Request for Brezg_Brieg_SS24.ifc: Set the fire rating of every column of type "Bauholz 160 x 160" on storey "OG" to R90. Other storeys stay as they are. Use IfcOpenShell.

First a look at what the model holds.

```python
import ifcopenshell
import ifcopenshell.util.element

model = ifcopenshell.open("Brezg_Brieg_SS24.ifc")
print(model.schema)
storey = next(s for s in model.by_type("IfcBuildingStorey") if s.Name == "OG")
columns = [e for e in ifcopenshell.util.element.get_decomposition(storey) if e.is_a("IfcColumn")]
seen = {}
for e in columns:
    element_type = ifcopenshell.util.element.get_type(e)
    key = (element_type.Name if element_type != e and element_type else None, ifcopenshell.util.element.get_pset(e, "Pset_ColumnCommon", "FireRating"))
    seen[key] = seen.get(key, 0) + 1
for (name, value), count in sorted(seen.items(), key=str):
    print(count, "x", name, "|", value)
```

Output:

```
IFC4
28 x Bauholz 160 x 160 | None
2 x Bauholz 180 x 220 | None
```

```python
import ifcopenshell
import ifcopenshell.api.pset
import ifcopenshell.util.element

model = ifcopenshell.open("Brezg_Brieg_SS24.ifc")

storey = next(s for s in model.by_type("IfcBuildingStorey") if s.Name == "OG")
columns = [e for e in ifcopenshell.util.element.get_decomposition(storey) if e.is_a("IfcColumn")]

count = 0
for e in columns:
    element_type = ifcopenshell.util.element.get_type(e)
    if element_type in (None, e) or element_type.Name != "Bauholz 160 x 160":
        continue
    # add_pset returns the element's existing set when there is one.
    pset = ifcopenshell.api.pset.add_pset(model, product=e, name="Pset_ColumnCommon")
    ifcopenshell.api.pset.edit_pset(model, pset=pset, properties={"FireRating": "R90"})
    count += 1

print(count, "columns updated")

model.write("Brezg_Brieg_SS24-out.ifc")
```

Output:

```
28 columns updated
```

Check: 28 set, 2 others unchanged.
